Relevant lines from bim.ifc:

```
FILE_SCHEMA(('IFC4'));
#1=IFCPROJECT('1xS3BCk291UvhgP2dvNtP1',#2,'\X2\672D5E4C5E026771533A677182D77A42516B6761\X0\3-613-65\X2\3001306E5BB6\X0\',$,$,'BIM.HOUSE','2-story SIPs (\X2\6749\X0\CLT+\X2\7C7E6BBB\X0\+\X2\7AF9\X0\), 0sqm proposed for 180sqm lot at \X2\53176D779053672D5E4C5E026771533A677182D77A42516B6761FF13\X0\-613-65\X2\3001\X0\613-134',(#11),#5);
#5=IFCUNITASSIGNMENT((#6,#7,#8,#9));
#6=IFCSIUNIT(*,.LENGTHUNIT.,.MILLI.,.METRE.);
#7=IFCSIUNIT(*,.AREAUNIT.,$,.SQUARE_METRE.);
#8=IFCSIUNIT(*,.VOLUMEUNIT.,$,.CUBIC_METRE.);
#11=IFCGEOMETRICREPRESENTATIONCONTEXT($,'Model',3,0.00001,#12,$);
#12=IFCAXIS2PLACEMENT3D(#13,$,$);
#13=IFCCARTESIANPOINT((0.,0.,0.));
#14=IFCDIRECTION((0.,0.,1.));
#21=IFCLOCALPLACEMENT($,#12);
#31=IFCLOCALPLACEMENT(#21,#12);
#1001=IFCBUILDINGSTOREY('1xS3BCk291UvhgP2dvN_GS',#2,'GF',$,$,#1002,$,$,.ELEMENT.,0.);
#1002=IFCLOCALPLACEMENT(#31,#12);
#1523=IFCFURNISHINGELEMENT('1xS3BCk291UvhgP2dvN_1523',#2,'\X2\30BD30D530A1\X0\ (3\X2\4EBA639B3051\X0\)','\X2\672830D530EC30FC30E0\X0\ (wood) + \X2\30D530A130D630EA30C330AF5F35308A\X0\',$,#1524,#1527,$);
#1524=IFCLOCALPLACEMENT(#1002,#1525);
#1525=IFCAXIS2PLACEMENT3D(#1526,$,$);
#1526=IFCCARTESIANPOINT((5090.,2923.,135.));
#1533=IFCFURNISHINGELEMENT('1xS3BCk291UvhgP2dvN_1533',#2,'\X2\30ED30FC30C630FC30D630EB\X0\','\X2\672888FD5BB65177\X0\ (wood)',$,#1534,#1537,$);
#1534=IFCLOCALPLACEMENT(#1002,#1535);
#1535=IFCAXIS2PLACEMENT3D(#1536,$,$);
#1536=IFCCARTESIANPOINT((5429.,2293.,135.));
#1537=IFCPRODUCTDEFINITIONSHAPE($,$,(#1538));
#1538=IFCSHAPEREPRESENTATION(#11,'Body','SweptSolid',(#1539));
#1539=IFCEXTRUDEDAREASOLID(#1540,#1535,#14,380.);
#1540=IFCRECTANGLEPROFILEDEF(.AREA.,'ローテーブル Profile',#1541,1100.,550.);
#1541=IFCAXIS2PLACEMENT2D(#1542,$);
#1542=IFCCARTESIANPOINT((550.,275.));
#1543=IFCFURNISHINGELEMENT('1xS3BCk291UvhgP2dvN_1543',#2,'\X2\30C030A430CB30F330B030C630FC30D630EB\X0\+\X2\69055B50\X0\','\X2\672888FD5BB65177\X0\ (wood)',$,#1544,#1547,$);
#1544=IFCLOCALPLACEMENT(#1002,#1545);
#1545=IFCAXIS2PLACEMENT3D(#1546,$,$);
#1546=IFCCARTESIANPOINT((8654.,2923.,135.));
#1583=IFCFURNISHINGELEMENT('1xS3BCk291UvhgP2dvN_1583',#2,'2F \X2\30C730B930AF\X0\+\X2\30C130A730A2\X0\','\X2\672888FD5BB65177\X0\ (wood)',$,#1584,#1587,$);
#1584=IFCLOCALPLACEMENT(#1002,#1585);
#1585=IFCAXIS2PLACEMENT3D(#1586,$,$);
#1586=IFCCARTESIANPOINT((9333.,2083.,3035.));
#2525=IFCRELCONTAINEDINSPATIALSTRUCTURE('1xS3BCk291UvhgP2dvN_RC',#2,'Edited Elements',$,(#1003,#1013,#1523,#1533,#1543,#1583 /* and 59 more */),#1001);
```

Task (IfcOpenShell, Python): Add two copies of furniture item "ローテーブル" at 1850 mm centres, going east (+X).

```python
import numpy as np
import ifcopenshell
import ifcopenshell.api.geometry
import ifcopenshell.api.root
import ifcopenshell.util.element
import ifcopenshell.util.placement
import ifcopenshell.util.unit

model = ifcopenshell.open("bim.ifc")
unit_scale = ifcopenshell.util.unit.calculate_unit_scale(model)


def reuse_history(source, copy):
    """copy_class also copies each property set's owner history, people and application; keep the originals."""
    for rel in copy.IsDefinedBy:
        if rel.is_a("IfcRelDefinesByProperties") and (history := rel.RelatingPropertyDefinition.OwnerHistory):
            rel.RelatingPropertyDefinition.OwnerHistory = source.OwnerHistory
            ifcopenshell.util.element.remove_deep2(model, history)


source = model.by_guid("1xS3BCk291UvhgP2dvN_1533")
base = ifcopenshell.util.placement.get_local_placement(source.ObjectPlacement)
step = np.array([1.0, 0.0, 0.0]) * 1.85 / unit_scale

for i in range(1, 3):
    copy = ifcopenshell.api.root.copy_class(model, product=source)
    copy.Representation = ifcopenshell.util.element.copy_deep(
        model, source.Representation, exclude=["IfcGeometricRepresentationContext", "IfcRepresentationMap"]
    )
    reuse_history(source, copy)
    matrix = base.copy()
    matrix[:3, 3] += i * step
    print("added at", matrix[:3, 3].round(3) + 0.0)
    ifcopenshell.api.geometry.edit_object_placement(model, product=copy, matrix=matrix, is_si=False)

model.write("bim_updated.ifc")
```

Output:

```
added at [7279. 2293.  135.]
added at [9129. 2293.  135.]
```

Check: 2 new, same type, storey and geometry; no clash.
